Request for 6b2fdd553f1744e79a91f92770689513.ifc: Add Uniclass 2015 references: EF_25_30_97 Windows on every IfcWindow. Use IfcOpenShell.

First a look at what the model holds.

```python
import ifcopenshell

model = ifcopenshell.open("6b2fdd553f1744e79a91f92770689513.ifc")
print(model.schema)
print("classifications:", [c.Name for c in model.by_type("IfcClassification")])
for ifc_class in ("IfcDoor", "IfcRoof", "IfcStair", "IfcWall", "IfcWindow"):
    print(ifc_class, len(model.by_type(ifc_class)))
```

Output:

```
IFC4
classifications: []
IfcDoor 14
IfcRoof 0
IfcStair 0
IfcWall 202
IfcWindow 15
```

```python
import ifcopenshell
import ifcopenshell.api.classification

model = ifcopenshell.open("6b2fdd553f1744e79a91f92770689513.ifc")

system = ifcopenshell.api.classification.add_classification(model, classification="Uniclass 2015")

codes = {
    "IfcWindow": ("EF_25_30_97", "Windows"),
}
for ifc_class, (code, name) in codes.items():
    products = model.by_type(ifc_class)
    ifcopenshell.api.classification.add_reference(
        model, products=products, classification=system, identification=code, name=name
    )
    print(code, len(products))

model.write("6b2fdd553f1744e79a91f92770689513_rev.ifc")
```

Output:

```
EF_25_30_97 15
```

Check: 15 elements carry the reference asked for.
